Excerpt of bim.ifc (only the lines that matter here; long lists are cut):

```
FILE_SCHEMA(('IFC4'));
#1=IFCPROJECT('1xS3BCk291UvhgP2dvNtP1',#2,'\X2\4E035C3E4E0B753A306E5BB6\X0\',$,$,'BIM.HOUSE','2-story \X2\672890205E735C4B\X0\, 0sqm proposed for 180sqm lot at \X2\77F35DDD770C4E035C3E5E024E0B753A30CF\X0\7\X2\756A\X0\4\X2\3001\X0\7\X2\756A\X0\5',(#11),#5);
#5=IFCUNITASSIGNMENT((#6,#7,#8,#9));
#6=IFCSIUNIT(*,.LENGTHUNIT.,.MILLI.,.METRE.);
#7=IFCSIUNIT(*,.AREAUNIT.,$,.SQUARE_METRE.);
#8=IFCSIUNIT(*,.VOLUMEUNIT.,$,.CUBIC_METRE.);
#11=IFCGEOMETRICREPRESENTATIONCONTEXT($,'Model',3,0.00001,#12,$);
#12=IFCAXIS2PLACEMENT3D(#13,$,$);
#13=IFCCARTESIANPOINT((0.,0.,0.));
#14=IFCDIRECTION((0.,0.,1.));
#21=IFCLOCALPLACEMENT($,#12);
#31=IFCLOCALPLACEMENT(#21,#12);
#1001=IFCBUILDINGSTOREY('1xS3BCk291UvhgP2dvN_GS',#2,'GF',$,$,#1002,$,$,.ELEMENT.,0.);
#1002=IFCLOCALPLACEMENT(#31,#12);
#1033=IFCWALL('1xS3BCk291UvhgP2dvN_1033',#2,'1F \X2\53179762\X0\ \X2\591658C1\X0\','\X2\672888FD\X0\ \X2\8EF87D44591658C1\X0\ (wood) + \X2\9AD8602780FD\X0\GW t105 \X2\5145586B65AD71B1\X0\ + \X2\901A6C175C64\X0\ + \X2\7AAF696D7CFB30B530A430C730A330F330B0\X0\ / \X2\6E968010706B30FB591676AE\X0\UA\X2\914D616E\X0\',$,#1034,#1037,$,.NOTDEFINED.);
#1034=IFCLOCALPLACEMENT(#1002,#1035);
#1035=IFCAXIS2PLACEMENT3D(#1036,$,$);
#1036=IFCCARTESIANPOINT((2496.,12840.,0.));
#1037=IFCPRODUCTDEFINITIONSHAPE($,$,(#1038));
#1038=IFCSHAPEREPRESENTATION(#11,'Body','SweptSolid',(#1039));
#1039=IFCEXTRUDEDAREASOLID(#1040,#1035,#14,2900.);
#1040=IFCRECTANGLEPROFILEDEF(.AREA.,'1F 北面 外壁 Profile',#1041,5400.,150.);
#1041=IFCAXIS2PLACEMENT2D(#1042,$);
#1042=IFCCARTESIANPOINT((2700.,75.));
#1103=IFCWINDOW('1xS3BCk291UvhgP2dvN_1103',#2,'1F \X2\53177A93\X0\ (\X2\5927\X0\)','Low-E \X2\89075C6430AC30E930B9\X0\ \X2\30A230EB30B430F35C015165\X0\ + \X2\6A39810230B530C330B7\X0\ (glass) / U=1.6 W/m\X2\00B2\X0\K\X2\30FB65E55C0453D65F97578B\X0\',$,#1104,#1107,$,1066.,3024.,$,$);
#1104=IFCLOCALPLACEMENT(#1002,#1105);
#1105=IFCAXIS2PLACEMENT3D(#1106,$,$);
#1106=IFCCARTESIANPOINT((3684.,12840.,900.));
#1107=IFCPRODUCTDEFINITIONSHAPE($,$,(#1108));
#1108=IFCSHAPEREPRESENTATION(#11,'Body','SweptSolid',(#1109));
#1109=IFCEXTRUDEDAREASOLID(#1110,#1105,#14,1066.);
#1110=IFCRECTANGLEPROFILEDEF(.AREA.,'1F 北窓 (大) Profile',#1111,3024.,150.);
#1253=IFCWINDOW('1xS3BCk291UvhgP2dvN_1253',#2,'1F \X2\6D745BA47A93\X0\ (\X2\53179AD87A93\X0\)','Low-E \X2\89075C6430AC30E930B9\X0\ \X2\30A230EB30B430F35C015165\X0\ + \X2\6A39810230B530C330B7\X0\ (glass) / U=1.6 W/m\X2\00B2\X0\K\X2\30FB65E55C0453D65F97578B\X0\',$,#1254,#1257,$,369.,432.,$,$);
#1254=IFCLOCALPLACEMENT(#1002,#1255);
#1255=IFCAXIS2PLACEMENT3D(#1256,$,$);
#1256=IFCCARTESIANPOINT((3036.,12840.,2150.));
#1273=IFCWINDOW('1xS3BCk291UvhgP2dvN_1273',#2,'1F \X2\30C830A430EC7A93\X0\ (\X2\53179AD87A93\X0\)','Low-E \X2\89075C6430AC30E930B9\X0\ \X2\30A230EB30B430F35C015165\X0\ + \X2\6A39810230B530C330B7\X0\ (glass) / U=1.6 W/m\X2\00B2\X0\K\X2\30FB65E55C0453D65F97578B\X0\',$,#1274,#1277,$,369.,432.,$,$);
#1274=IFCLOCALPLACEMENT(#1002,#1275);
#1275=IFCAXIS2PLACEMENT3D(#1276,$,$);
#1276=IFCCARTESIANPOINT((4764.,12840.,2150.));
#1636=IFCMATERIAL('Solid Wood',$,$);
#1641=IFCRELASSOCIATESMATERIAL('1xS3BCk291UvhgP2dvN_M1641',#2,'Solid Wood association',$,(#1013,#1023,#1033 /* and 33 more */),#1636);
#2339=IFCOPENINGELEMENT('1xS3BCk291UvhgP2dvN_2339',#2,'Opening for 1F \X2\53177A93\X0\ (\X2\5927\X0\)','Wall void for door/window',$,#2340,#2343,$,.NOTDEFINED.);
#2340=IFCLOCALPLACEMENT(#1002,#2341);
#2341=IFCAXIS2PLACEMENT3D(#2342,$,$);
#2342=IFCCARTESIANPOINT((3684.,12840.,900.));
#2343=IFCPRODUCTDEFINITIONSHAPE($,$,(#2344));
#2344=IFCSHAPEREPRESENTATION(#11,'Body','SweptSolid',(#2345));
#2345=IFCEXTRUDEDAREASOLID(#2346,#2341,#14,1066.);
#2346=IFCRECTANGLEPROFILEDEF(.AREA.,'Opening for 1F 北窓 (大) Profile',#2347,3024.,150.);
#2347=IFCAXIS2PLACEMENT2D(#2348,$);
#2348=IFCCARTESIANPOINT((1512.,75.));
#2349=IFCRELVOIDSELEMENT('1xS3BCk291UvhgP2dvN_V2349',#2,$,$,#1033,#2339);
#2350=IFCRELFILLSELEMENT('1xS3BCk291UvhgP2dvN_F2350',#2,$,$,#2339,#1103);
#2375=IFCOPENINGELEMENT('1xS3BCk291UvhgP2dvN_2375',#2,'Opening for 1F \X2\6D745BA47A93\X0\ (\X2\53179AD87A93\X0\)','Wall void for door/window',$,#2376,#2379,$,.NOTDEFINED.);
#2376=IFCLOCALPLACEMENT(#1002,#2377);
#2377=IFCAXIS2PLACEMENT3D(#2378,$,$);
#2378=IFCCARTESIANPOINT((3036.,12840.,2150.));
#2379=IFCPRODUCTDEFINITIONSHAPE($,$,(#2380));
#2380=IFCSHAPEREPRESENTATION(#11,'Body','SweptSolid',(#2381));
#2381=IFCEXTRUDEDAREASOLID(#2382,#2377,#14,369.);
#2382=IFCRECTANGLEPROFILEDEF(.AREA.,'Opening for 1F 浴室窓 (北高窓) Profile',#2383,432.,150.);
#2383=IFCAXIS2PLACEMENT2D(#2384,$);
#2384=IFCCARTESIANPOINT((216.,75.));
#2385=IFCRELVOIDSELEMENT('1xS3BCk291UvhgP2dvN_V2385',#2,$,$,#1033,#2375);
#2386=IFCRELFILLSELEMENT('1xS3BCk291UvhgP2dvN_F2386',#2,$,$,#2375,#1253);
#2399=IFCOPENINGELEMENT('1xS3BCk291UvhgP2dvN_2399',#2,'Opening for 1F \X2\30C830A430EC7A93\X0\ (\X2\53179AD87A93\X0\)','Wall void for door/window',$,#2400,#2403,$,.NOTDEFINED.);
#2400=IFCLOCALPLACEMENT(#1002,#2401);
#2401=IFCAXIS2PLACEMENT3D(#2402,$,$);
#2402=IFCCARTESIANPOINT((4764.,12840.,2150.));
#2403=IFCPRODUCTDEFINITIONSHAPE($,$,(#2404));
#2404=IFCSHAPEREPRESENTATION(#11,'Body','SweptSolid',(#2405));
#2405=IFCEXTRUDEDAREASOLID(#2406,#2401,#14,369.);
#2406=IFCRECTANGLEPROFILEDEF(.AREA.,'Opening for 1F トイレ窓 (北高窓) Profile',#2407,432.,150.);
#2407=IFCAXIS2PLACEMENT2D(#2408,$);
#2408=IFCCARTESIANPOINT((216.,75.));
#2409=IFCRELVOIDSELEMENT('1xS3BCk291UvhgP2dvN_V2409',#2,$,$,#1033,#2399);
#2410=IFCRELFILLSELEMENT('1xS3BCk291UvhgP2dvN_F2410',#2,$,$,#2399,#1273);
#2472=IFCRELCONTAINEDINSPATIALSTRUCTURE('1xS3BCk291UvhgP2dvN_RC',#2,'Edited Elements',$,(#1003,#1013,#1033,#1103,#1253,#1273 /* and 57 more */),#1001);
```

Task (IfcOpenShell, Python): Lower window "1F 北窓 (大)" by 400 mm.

```python
import numpy as np
import ifcopenshell
import ifcopenshell.api.geometry
import ifcopenshell.util.placement
import ifcopenshell.util.unit

model = ifcopenshell.open("bim.ifc")
unit_scale = ifcopenshell.util.unit.calculate_unit_scale(model)

window = model.by_guid("1xS3BCk291UvhgP2dvN_1103")
opening = window.FillsVoids[0].RelatingOpeningElement
dz = -0.4 / unit_scale

shift = np.array([0.0, 0.0, dz])
# The window is not placed relative to its opening, so move both.
for product in (opening, window):
    matrix = ifcopenshell.util.placement.get_local_placement(product.ObjectPlacement)
    matrix[:3, 3] += shift
    ifcopenshell.api.geometry.edit_object_placement(model, product=product, matrix=matrix, is_si=False)

print(f"moved by {dz * unit_scale:+.3f} m")

model.write("bim-out.ifc")
```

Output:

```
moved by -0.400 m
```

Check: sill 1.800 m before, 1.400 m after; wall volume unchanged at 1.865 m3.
